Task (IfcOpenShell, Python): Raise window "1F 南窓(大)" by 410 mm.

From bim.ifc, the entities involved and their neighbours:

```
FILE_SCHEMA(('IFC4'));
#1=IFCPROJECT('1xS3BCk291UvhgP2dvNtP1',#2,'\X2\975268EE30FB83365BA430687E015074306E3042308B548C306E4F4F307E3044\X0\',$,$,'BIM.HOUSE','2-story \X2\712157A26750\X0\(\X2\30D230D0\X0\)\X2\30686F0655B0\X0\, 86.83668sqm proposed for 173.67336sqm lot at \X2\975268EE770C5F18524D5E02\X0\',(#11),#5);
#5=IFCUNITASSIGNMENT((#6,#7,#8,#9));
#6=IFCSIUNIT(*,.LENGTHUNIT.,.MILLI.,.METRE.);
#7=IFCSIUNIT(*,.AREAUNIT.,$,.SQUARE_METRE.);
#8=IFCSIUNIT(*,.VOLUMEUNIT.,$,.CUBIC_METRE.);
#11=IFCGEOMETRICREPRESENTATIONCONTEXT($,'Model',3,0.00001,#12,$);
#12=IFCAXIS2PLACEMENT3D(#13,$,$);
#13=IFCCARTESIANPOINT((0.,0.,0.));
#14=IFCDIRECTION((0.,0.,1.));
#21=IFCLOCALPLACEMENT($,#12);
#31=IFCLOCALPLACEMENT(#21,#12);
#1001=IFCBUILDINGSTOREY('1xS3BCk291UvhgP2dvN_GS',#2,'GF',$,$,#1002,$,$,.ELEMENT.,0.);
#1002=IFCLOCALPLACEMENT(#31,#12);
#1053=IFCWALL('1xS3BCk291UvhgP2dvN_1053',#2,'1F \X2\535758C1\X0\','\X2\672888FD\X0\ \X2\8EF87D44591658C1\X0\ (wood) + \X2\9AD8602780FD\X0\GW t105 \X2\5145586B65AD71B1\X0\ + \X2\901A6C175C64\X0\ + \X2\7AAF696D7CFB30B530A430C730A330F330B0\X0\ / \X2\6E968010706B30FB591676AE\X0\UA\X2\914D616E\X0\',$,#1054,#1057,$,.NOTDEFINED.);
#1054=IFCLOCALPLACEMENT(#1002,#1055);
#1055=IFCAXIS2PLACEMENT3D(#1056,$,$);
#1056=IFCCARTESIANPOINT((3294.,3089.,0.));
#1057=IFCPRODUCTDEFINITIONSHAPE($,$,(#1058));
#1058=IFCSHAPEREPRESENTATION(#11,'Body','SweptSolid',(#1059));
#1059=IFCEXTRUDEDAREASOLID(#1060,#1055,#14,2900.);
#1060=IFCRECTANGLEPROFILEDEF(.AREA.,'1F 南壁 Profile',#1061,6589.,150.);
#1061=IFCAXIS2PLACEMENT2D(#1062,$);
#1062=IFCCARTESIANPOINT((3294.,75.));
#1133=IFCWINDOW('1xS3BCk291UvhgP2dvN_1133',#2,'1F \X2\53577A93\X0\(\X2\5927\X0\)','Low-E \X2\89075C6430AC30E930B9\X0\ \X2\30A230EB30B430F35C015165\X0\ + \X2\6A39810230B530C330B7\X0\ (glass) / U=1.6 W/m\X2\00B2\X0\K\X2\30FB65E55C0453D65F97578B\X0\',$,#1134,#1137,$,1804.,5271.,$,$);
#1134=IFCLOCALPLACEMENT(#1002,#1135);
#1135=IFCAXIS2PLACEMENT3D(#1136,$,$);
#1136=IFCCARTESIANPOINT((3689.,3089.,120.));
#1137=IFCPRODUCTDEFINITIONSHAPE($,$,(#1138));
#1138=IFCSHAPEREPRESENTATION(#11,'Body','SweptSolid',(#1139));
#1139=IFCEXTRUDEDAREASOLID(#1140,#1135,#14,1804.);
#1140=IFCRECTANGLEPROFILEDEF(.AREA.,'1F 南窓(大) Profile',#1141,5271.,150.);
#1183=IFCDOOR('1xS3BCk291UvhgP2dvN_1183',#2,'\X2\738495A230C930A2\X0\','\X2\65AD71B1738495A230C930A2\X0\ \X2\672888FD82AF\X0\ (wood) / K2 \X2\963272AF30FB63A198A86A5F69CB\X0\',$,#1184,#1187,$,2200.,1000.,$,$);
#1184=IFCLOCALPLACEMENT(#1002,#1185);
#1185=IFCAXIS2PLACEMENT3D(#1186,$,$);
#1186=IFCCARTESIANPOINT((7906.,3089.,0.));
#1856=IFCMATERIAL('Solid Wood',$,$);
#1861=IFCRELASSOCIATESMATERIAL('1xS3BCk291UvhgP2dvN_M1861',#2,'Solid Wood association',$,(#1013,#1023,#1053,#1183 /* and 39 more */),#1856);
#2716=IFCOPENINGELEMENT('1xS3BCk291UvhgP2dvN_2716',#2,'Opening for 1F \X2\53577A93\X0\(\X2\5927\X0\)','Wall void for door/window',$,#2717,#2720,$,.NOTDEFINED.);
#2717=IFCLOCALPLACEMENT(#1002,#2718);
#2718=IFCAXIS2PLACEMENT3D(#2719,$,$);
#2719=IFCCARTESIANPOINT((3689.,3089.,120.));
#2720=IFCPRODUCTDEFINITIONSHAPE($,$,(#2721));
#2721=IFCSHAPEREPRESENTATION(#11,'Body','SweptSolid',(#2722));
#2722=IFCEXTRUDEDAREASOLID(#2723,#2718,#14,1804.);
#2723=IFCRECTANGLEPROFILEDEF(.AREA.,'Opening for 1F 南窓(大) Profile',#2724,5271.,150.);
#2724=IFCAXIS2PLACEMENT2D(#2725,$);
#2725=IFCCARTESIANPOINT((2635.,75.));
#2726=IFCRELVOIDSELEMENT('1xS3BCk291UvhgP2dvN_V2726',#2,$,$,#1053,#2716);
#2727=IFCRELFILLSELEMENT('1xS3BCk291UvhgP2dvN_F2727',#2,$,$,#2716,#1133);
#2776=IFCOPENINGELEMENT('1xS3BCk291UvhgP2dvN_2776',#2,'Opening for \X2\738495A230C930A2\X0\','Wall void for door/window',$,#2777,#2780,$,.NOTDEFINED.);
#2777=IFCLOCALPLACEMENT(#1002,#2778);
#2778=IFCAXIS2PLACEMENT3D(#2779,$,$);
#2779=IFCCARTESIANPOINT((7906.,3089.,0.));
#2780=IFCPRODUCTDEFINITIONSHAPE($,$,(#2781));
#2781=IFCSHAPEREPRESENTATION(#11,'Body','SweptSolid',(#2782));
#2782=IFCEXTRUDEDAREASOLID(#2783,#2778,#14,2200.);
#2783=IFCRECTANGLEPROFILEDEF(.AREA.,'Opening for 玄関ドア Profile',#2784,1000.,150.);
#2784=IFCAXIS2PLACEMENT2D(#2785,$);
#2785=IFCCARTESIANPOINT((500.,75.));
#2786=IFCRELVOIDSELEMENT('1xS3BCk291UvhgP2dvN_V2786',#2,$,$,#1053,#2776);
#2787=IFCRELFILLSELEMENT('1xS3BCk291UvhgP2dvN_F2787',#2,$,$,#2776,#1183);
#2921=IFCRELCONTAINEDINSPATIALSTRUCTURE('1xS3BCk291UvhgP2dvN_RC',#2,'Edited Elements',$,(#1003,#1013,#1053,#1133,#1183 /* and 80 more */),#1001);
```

```python
import numpy as np
import ifcopenshell
import ifcopenshell.api.geometry
import ifcopenshell.util.placement
import ifcopenshell.util.unit

model = ifcopenshell.open("bim.ifc")
unit_scale = ifcopenshell.util.unit.calculate_unit_scale(model)

window = model.by_guid("1xS3BCk291UvhgP2dvN_1133")
opening = window.FillsVoids[0].RelatingOpeningElement
dz = 0.41 / unit_scale

shift = np.array([0.0, 0.0, dz])
# The window is not placed relative to its opening, so move both.
for product in (opening, window):
    matrix = ifcopenshell.util.placement.get_local_placement(product.ObjectPlacement)
    matrix[:3, 3] += shift
    ifcopenshell.api.geometry.edit_object_placement(model, product=product, matrix=matrix, is_si=False)

print(f"moved by {dz * unit_scale:+.3f} m")

model.write("bim_edited.ifc")
```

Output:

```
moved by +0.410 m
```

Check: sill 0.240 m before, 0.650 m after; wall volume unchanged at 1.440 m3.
